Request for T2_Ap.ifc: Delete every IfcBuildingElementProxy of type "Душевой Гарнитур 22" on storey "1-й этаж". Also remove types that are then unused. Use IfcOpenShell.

First a look at what the model holds.

```python
import ifcopenshell
import ifcopenshell.util.element

model = ifcopenshell.open("T2_Ap.ifc")
print(model.schema)
storey = next(s for s in model.by_type("IfcBuildingStorey") if s.Name == "1-й этаж")
proxies = [e for e in ifcopenshell.util.element.get_decomposition(storey) if e.is_a("IfcBuildingElementProxy")]
seen = {}
for e in proxies:
    element_type = ifcopenshell.util.element.get_type(e)
    name = element_type.Name if element_type not in (None, e) else None
    seen[name] = seen.get(name, 0) + 1
for name, count in sorted(seen.items(), key=str):
    print(count, "x", name)
```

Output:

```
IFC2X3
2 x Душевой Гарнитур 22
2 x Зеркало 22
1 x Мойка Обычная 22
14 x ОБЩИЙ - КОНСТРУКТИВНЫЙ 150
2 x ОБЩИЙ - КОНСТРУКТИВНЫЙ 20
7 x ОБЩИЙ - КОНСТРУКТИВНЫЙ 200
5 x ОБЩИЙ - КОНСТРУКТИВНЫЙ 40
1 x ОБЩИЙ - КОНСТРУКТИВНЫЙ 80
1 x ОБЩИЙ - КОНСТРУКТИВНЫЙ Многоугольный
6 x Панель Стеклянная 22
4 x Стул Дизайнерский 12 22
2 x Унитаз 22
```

```python
import ifcopenshell
import ifcopenshell.api.root
import ifcopenshell.util.element

model = ifcopenshell.open("T2_Ap.ifc")

storey = next(s for s in model.by_type("IfcBuildingStorey") if s.Name == "1-й этаж")
proxies = [e for e in ifcopenshell.util.element.get_decomposition(storey) if e.is_a("IfcBuildingElementProxy")]
targets = [e for e in proxies if (t := ifcopenshell.util.element.get_type(e)) not in (None, e) and t.Name == "Душевой Гарнитур 22"]
types = {ifcopenshell.util.element.get_type(e) for e in targets} - {None, *targets}

for e in targets:
    ifcopenshell.api.root.remove_product(model, product=e)
print(len(targets), "removed")

unused = [t for t in types if not ifcopenshell.util.element.get_types(t)]
for t in unused:
    ifcopenshell.api.root.remove_product(model, product=t)
print(len(unused), "unused types removed")

model.write("T2_Ap-out.ifc")
```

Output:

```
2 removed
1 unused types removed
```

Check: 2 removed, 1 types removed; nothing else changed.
